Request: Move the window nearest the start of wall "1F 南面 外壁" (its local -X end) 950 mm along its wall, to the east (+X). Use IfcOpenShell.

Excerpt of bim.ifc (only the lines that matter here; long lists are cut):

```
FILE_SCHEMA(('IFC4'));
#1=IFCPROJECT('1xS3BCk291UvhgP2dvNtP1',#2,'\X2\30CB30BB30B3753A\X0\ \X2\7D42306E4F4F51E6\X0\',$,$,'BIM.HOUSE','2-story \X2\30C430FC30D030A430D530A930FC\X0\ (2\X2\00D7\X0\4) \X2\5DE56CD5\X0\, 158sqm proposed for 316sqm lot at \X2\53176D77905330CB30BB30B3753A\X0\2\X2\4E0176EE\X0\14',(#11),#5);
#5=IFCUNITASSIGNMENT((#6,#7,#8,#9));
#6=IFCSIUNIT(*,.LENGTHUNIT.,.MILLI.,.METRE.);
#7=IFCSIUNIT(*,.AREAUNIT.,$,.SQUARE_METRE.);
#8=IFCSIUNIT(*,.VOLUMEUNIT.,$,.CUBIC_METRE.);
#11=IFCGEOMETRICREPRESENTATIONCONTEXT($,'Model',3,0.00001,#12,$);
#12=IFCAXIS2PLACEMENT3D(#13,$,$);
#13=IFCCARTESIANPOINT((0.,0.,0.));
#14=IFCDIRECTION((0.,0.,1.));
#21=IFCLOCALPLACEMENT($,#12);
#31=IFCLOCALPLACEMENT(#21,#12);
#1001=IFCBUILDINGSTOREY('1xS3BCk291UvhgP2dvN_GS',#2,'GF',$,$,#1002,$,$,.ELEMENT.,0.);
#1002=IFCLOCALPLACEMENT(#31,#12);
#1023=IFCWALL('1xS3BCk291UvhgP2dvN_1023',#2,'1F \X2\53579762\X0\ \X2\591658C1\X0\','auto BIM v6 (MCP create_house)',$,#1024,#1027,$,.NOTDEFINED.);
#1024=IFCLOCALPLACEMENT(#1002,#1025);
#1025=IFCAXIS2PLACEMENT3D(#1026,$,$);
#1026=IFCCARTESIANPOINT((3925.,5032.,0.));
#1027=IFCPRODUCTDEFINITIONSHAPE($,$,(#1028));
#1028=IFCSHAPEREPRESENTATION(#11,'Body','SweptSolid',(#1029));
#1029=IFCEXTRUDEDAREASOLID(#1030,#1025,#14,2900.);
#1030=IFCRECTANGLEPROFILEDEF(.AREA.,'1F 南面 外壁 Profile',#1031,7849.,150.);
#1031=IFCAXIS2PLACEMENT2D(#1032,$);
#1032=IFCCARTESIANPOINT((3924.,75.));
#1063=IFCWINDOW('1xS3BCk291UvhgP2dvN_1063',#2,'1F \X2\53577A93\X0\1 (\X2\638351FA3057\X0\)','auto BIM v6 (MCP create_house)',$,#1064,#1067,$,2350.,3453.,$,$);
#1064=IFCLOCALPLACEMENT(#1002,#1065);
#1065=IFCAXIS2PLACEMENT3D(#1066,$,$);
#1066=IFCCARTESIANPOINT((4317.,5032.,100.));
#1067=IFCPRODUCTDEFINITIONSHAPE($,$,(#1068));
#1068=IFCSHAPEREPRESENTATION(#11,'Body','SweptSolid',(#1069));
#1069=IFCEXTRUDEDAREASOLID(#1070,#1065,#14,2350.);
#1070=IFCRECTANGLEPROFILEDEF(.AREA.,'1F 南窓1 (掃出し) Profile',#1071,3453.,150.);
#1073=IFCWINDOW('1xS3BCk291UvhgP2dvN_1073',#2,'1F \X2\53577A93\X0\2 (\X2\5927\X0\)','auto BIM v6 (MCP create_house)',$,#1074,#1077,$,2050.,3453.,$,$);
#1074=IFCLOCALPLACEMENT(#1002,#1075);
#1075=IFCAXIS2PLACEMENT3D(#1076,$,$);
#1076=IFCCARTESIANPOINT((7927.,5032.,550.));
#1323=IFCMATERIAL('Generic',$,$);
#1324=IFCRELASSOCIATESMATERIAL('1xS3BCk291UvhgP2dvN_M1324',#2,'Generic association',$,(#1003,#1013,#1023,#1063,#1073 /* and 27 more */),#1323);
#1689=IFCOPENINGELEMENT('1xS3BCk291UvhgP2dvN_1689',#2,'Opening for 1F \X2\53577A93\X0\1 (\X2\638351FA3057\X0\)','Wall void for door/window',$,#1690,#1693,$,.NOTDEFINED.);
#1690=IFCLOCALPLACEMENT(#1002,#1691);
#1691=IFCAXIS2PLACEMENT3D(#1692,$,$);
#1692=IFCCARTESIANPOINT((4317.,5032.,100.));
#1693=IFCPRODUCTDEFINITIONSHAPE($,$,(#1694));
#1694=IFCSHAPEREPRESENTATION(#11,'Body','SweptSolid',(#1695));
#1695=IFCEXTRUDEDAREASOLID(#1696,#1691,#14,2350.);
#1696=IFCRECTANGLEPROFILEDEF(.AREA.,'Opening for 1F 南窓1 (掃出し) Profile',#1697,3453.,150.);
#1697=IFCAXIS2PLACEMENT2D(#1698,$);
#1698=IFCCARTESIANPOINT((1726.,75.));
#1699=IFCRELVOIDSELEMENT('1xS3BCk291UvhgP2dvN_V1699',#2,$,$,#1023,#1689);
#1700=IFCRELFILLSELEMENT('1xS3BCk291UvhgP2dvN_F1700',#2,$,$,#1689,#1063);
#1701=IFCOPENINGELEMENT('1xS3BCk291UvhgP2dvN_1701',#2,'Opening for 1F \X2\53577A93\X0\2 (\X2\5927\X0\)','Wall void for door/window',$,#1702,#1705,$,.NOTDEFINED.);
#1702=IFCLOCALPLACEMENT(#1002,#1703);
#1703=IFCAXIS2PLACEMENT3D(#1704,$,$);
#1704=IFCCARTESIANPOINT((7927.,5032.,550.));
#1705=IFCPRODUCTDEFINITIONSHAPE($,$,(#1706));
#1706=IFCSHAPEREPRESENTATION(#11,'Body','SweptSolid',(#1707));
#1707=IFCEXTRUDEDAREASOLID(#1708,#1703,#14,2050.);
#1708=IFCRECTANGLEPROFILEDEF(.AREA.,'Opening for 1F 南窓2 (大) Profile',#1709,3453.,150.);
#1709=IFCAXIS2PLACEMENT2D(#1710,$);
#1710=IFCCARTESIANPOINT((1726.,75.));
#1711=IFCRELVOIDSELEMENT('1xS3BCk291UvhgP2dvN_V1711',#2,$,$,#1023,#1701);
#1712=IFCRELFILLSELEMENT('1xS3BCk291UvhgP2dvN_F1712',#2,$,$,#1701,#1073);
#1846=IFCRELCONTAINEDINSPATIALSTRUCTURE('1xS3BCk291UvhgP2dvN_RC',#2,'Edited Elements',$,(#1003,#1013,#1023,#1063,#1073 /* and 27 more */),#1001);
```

```python
import ifcopenshell
import ifcopenshell.api.geometry
import ifcopenshell.util.placement
import ifcopenshell.util.unit

model = ifcopenshell.open("bim.ifc")
unit_scale = ifcopenshell.util.unit.calculate_unit_scale(model)

window = model.by_id(1063)
opening = window.FillsVoids[0].RelatingOpeningElement
wall = opening.VoidsElements[0].RelatingBuildingElement

wall_matrix = ifcopenshell.util.placement.get_local_placement(wall.ObjectPlacement)
shift = wall_matrix[:3, 0] * 0.95 / unit_scale
before = ifcopenshell.util.placement.get_local_placement(window.ObjectPlacement)[:3, 3].copy()

# The window is not placed relative to its opening, so move both.
for product in (opening, window):
    matrix = ifcopenshell.util.placement.get_local_placement(product.ObjectPlacement)
    matrix[:3, 3] += shift
    ifcopenshell.api.geometry.edit_object_placement(model, product=product, matrix=matrix, is_si=False)

after = ifcopenshell.util.placement.get_local_placement(window.ObjectPlacement)[:3, 3]
print("window moved by", (after - before).round(3) + 0.0)

model.write("bim_v2.ifc")
```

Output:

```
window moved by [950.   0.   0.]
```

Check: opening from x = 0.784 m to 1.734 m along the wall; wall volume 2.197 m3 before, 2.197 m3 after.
